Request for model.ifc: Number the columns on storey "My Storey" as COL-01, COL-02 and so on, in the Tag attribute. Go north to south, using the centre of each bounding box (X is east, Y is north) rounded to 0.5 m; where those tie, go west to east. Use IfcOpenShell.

First a look at what the model holds.

```python
import ifcopenshell
import ifcopenshell.util.element
import ifcopenshell.util.placement

model = ifcopenshell.open("model.ifc")
print(model.schema)
storey = next(s for s in model.by_type("IfcBuildingStorey") if s.Name == "My Storey")
columns = [e for e in ifcopenshell.util.element.get_decomposition(storey) if e.is_a("IfcColumn")]
for e in sorted(columns, key=lambda e: e.id()):
    origin = ifcopenshell.util.placement.get_local_placement(e.ObjectPlacement)[:3, 3]
    print(e.id(), e.Tag, e.Name, origin.round(2) + 0.0, sep=" | ")
```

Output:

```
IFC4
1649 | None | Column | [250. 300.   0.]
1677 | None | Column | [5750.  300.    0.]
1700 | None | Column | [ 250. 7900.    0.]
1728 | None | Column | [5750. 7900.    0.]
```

```python
import ifcopenshell
import ifcopenshell.geom
import ifcopenshell.util.element
import ifcopenshell.util.shape

model = ifcopenshell.open("model.ifc")
settings = ifcopenshell.geom.settings()
settings.set("use-world-coords", True)


def centre(element):
    shape = ifcopenshell.geom.create_shape(settings, element)
    return ifcopenshell.util.shape.get_bbox_centroid(shape.geometry)


storey = next(s for s in model.by_type("IfcBuildingStorey") if s.Name == "My Storey")
columns = [e for e in ifcopenshell.util.element.get_decomposition(storey) if e.is_a("IfcColumn")]

# Insertion points can sit at a corner or the storey origin, so sort by the geometry (in metres).
centres = {e: centre(e) for e in columns}
columns.sort(key=lambda e: (-round(centres[e][1] / 0.5), centres[e][0]))

for i, e in enumerate(columns, start=1):
    number = f"COL-{i:02d}"
    e.Tag = number
    print(e.id(), number)

model.write("model_updated.ifc")
```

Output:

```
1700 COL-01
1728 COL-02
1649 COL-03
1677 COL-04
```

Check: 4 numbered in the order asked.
